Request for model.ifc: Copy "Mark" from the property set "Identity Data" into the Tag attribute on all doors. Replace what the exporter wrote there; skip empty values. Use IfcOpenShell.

First a look at what the model holds.

```python
import ifcopenshell
import ifcopenshell.util.element

model = ifcopenshell.open("model.ifc")
print(model.schema)
doors = model.by_type("IfcDoor")
print(len(doors), "doors")
for e in doors[:8]:
    source = ifcopenshell.util.element.get_pset(e, "Identity Data", "Mark")
    target = e.Tag
    print(e.id(), repr(source), repr(target), sep=" | ")
```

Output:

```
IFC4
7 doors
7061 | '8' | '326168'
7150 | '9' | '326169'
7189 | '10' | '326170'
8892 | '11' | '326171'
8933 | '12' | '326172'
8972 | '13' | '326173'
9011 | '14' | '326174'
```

```python
import ifcopenshell
import ifcopenshell.util.element

model = ifcopenshell.open("model.ifc")

count = 0
for e in model.by_type("IfcDoor"):
    value = ifcopenshell.util.element.get_pset(e, "Identity Data", "Mark")
    current = e.Tag
    if not value or not value.strip() or current == value:
        continue
    e.Tag = value
    count += 1

print(count, "doors updated")

model.write("model_edited.ifc")
```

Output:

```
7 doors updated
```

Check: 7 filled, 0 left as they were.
